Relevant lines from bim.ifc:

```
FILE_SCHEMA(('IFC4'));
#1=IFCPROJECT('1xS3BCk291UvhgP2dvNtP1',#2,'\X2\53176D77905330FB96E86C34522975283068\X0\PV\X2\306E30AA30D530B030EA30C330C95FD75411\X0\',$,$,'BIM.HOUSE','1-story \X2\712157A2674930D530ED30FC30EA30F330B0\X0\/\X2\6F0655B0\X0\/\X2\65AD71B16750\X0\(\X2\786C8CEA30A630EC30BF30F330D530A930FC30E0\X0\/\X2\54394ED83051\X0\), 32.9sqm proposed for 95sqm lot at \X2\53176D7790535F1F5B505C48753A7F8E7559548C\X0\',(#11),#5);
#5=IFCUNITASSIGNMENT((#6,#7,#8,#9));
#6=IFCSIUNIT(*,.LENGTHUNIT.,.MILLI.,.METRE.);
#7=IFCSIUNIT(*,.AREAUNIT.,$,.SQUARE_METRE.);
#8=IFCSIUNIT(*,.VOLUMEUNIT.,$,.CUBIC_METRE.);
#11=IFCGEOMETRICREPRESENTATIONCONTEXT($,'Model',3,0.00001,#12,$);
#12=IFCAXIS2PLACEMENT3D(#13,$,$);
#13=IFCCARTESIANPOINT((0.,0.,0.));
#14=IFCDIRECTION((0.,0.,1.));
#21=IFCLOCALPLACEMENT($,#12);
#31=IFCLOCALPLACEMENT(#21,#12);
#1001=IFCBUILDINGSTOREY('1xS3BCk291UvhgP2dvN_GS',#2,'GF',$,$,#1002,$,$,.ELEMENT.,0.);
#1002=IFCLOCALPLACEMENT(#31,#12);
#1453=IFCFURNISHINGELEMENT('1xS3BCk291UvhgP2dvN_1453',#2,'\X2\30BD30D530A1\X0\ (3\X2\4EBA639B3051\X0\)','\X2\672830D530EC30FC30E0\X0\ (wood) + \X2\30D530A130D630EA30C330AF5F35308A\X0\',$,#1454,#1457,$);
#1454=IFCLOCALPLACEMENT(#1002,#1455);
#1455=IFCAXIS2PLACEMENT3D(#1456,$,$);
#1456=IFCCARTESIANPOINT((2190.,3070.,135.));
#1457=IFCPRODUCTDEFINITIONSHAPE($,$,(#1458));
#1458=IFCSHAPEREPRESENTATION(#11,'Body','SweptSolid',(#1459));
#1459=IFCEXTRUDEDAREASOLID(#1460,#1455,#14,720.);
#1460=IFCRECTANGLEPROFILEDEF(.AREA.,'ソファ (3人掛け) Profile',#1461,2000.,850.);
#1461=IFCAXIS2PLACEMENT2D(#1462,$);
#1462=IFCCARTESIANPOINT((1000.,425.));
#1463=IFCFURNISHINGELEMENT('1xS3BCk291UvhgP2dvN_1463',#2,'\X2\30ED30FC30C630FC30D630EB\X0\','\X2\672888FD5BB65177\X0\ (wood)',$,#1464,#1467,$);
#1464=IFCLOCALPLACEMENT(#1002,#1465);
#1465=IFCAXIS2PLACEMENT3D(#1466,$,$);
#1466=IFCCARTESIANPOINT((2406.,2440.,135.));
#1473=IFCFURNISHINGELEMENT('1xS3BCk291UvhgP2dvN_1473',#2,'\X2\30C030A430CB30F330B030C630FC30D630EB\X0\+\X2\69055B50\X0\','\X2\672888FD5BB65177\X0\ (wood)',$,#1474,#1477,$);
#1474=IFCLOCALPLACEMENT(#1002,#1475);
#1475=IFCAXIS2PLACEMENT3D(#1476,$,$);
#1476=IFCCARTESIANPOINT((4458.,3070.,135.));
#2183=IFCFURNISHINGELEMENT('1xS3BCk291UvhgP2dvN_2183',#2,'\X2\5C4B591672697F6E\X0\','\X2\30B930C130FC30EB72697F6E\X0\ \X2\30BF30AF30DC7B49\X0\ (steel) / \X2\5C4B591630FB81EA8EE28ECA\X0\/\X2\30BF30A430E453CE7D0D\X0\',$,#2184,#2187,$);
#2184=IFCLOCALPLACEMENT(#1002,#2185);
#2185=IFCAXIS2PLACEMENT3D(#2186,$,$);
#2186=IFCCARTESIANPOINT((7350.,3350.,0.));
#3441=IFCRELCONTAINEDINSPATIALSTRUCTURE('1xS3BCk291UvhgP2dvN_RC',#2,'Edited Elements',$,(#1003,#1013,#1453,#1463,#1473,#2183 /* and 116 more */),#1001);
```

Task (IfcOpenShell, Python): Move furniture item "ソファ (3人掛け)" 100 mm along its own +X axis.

```python
import ifcopenshell
import ifcopenshell.api.geometry
import ifcopenshell.util.placement

model = ifcopenshell.open("bim.ifc")

item = model.by_guid("1xS3BCk291UvhgP2dvN_1453")
matrix = ifcopenshell.util.placement.get_local_placement(item.ObjectPlacement)
matrix[:3, 3] += matrix[:3, 0] * 100.0
ifcopenshell.api.geometry.edit_object_placement(model, product=item, matrix=matrix, is_si=False)

print(ifcopenshell.util.placement.get_local_placement(item.ObjectPlacement).round(3) + 0.0)

model.write("bim_rev.ifc")
```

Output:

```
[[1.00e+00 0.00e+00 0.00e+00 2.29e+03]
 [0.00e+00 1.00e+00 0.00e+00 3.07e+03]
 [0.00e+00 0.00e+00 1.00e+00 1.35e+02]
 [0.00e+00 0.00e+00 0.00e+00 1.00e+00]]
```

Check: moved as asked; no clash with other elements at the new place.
